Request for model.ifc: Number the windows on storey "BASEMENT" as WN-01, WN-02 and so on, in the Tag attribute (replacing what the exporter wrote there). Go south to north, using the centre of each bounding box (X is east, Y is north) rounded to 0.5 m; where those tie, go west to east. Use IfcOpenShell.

First a look at what the model holds.

```python
import ifcopenshell
import ifcopenshell.util.element
import ifcopenshell.util.placement

model = ifcopenshell.open("model.ifc")
print(model.schema)
storey = next(s for s in model.by_type("IfcBuildingStorey") if s.Name == "BASEMENT")
windows = [e for e in ifcopenshell.util.element.get_decomposition(storey) if e.is_a("IfcWindow")]
for e in sorted(windows, key=lambda e: e.id()):
    origin = ifcopenshell.util.placement.get_local_placement(e.ObjectPlacement)[:3, 3]
    print(e.id(), e.Tag, e.Name, origin.round(2) + 0.0, sep=" | ")
```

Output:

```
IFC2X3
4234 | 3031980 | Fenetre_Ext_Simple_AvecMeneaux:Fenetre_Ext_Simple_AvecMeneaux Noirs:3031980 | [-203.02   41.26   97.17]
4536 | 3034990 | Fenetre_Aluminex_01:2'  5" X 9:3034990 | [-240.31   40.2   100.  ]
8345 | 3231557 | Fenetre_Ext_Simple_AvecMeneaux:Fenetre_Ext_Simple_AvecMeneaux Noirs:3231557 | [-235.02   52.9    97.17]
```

```python
import ifcopenshell
import ifcopenshell.geom
import ifcopenshell.util.element
import ifcopenshell.util.shape

model = ifcopenshell.open("model.ifc")
settings = ifcopenshell.geom.settings()
settings.set("use-world-coords", True)


def centre(element):
    shape = ifcopenshell.geom.create_shape(settings, element)
    return ifcopenshell.util.shape.get_bbox_centroid(shape.geometry)


storey = next(s for s in model.by_type("IfcBuildingStorey") if s.Name == "BASEMENT")
windows = [e for e in ifcopenshell.util.element.get_decomposition(storey) if e.is_a("IfcWindow")]

# Insertion points can sit at a corner or the storey origin, so sort by the geometry (in metres).
centres = {e: centre(e) for e in windows}
windows.sort(key=lambda e: (round(centres[e][1] / 0.5), centres[e][0]))

for i, e in enumerate(windows, start=1):
    number = f"WN-{i:02d}"
    e.Tag = number
    print(e.id(), number)

model.write("model_v2.ifc")
```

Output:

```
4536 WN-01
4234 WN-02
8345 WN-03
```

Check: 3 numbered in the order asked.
